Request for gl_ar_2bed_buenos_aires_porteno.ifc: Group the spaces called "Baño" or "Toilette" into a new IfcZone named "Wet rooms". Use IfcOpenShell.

First a look at what the model holds.

```python
import ifcopenshell

model = ifcopenshell.open("gl_ar_2bed_buenos_aires_porteno.ifc")
print(model.schema)
seen = {}
for space in model.by_type("IfcSpace"):
    seen[space.LongName] = seen.get(space.LongName, 0) + 1
for name, count in sorted(seen.items(), key=str):
    print(count, "x", name)
print("zones:", [z.Name for z in model.by_type("IfcZone")][:20])
```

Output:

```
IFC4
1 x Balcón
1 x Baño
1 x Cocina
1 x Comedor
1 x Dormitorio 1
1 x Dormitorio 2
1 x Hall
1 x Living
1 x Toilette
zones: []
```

```python
import ifcopenshell
import ifcopenshell.api.group
import ifcopenshell.api.root

model = ifcopenshell.open("gl_ar_2bed_buenos_aires_porteno.ifc")

names = {"Baño", "Toilette"}
spaces = [s for s in model.by_type("IfcSpace") if s.LongName in names]

zone = ifcopenshell.api.root.create_entity(model, ifc_class="IfcZone", name="Wet rooms")
ifcopenshell.api.group.assign_group(model, products=spaces, group=zone)
print(len(spaces), "spaces in", zone.Name)

model.write("gl_ar_2bed_buenos_aires_porteno_rev.ifc")
```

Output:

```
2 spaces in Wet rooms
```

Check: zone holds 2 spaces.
